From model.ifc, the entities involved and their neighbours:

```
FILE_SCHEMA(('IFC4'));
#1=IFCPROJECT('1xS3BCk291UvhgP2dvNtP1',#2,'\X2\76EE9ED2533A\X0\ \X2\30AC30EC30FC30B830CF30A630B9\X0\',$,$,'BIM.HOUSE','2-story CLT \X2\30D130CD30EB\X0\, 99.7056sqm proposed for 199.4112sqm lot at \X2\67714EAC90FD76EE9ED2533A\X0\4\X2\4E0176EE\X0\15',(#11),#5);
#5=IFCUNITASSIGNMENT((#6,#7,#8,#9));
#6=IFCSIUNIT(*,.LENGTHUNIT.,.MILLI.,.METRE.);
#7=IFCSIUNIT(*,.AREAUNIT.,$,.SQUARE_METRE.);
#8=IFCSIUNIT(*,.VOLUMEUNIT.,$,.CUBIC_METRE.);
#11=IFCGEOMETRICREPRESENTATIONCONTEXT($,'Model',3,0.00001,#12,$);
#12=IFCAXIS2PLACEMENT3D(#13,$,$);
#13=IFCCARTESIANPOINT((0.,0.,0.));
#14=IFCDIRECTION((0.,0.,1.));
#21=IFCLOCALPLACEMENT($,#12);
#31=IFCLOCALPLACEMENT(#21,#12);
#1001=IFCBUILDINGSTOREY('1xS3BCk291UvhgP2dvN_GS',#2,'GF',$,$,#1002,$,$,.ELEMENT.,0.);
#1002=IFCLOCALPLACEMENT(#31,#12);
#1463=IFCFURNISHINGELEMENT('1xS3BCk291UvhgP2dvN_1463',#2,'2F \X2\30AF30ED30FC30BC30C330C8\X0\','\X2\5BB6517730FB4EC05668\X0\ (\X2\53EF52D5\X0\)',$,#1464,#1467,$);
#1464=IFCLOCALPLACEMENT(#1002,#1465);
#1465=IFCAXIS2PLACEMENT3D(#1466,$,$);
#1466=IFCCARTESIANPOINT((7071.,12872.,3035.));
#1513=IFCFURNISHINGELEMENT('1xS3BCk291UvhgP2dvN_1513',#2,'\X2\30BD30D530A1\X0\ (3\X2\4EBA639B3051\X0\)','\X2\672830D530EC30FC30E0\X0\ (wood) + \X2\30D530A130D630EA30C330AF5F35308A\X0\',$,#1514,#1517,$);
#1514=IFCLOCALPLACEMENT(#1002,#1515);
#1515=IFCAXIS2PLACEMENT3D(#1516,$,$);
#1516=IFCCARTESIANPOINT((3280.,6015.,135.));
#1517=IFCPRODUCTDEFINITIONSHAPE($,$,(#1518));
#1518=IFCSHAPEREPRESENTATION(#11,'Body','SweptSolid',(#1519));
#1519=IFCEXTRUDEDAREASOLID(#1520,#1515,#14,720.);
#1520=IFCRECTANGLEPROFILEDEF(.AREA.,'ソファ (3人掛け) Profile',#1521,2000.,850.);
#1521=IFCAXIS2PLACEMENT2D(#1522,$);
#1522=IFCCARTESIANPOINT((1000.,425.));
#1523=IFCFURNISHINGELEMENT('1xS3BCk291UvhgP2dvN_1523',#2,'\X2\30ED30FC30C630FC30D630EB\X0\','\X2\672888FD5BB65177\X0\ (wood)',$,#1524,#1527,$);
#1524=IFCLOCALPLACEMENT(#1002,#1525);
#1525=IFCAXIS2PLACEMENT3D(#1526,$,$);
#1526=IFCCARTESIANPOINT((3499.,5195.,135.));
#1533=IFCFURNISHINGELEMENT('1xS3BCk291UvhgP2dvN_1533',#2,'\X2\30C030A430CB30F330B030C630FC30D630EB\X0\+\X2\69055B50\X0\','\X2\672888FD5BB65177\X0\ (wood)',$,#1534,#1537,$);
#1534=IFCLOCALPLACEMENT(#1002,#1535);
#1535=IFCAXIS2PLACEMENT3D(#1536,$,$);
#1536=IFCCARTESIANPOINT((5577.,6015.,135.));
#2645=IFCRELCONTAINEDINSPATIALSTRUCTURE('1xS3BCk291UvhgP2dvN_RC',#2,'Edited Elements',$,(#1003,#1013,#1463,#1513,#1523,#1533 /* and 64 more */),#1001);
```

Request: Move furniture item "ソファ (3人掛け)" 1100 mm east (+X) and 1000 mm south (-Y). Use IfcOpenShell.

```python
import ifcopenshell
import ifcopenshell.api.geometry
import ifcopenshell.util.placement

model = ifcopenshell.open("model.ifc")

item = model.by_guid("1xS3BCk291UvhgP2dvN_1513")
matrix = ifcopenshell.util.placement.get_local_placement(item.ObjectPlacement)
matrix[0, 3] += 1100.0
matrix[1, 3] -= 1000.0
ifcopenshell.api.geometry.edit_object_placement(model, product=item, matrix=matrix, is_si=False)

print(ifcopenshell.util.placement.get_local_placement(item.ObjectPlacement).round(3) + 0.0)

model.write("model_rev.ifc")
```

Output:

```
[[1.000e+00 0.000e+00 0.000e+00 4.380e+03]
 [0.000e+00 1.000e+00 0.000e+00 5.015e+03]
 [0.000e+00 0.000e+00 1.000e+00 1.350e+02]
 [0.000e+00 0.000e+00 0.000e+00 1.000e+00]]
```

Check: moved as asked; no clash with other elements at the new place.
